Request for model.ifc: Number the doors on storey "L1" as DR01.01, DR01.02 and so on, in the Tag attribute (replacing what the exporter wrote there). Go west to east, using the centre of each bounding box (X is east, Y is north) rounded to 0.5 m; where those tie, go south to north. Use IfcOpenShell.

First a look at what the model holds.

```python
import ifcopenshell
import ifcopenshell.util.element
import ifcopenshell.util.placement

model = ifcopenshell.open("model.ifc")
print(model.schema)
storey = next(s for s in model.by_type("IfcBuildingStorey") if s.Name == "L1")
doors = [e for e in ifcopenshell.util.element.get_decomposition(storey) if e.is_a("IfcDoor")]
for e in sorted(doors, key=lambda e: e.id()):
    origin = ifcopenshell.util.placement.get_local_placement(e.ObjectPlacement)[:3, 3]
    print(e.id(), e.Tag, e.Name, origin.round(2) + 0.0, sep=" | ")
```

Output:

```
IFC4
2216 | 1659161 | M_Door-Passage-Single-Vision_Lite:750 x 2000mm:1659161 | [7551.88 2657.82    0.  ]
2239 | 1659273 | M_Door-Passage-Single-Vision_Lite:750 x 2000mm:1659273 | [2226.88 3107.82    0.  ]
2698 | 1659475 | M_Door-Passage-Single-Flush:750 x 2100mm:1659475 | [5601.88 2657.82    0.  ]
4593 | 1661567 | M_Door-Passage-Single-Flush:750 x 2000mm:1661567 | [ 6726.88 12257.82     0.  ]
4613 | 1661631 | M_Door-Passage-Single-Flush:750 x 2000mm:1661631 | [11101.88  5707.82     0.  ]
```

```python
import ifcopenshell
import ifcopenshell.geom
import ifcopenshell.util.element
import ifcopenshell.util.shape

model = ifcopenshell.open("model.ifc")
settings = ifcopenshell.geom.settings()
settings.set("use-world-coords", True)


def centre(element):
    shape = ifcopenshell.geom.create_shape(settings, element)
    return ifcopenshell.util.shape.get_bbox_centroid(shape.geometry)


storey = next(s for s in model.by_type("IfcBuildingStorey") if s.Name == "L1")
doors = [e for e in ifcopenshell.util.element.get_decomposition(storey) if e.is_a("IfcDoor")]

# Insertion points can sit at a corner or the storey origin, so sort by the geometry (in metres).
centres = {e: centre(e) for e in doors}
doors.sort(key=lambda e: (round(centres[e][0] / 0.5), centres[e][1]))

for i, e in enumerate(doors, start=1):
    number = f"DR01.{i:02d}"
    e.Tag = number
    print(e.id(), number)

model.write("model_v2.ifc")
```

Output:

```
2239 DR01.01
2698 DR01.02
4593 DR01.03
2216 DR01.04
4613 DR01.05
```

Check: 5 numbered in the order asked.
